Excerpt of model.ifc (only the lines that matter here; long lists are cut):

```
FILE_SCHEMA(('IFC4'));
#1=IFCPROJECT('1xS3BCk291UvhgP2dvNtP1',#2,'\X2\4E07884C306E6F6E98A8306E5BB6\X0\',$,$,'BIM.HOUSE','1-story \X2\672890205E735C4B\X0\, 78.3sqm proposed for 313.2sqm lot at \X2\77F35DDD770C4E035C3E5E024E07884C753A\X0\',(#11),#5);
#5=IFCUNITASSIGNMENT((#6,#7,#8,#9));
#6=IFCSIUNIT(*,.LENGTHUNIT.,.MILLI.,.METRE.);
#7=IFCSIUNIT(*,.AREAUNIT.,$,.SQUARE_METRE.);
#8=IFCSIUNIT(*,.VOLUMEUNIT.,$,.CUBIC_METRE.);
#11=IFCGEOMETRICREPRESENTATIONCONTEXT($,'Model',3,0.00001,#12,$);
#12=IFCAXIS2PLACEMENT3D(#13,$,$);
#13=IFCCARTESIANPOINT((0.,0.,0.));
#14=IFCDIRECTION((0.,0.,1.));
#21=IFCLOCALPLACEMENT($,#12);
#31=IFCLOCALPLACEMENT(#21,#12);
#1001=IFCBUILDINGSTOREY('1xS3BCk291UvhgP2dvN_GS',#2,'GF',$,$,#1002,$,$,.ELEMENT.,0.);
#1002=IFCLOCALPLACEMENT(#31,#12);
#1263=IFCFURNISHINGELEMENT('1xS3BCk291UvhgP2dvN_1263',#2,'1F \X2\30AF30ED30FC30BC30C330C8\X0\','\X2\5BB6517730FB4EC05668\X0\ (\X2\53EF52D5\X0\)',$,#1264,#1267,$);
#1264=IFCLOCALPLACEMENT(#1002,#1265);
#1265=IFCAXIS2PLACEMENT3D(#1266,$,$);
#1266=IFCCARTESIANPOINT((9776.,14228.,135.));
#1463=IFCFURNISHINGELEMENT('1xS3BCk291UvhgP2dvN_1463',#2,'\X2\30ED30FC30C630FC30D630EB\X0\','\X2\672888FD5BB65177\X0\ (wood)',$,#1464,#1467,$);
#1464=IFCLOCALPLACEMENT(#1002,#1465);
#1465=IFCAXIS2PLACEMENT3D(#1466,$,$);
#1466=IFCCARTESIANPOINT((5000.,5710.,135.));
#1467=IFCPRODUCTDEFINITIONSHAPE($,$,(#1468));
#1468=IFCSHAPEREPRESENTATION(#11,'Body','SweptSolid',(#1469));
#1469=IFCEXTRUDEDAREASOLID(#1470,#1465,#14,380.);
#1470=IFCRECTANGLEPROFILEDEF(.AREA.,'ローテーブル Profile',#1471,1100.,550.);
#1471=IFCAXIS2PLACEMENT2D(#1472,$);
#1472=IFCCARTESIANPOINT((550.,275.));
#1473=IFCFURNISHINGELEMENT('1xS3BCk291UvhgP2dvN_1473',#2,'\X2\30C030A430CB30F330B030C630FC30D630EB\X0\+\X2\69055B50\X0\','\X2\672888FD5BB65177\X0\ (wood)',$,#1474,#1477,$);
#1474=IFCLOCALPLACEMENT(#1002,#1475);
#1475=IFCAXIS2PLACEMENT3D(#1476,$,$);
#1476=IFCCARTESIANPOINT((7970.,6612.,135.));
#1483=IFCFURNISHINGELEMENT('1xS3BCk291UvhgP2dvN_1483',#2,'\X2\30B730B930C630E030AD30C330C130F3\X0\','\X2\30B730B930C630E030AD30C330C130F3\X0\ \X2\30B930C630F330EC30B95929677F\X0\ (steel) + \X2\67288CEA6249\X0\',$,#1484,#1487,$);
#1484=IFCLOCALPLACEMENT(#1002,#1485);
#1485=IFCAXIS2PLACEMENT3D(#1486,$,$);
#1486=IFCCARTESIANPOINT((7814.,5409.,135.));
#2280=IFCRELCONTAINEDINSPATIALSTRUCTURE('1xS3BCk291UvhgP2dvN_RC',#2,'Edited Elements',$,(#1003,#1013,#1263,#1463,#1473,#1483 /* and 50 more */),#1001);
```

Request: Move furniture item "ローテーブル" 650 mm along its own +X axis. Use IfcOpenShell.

```python
import ifcopenshell
import ifcopenshell.api.geometry
import ifcopenshell.util.placement

model = ifcopenshell.open("model.ifc")

item = model.by_guid("1xS3BCk291UvhgP2dvN_1463")
matrix = ifcopenshell.util.placement.get_local_placement(item.ObjectPlacement)
matrix[:3, 3] += matrix[:3, 0] * 650.0
ifcopenshell.api.geometry.edit_object_placement(model, product=item, matrix=matrix, is_si=False)

print(ifcopenshell.util.placement.get_local_placement(item.ObjectPlacement).round(3) + 0.0)

model.write("model-out.ifc")
```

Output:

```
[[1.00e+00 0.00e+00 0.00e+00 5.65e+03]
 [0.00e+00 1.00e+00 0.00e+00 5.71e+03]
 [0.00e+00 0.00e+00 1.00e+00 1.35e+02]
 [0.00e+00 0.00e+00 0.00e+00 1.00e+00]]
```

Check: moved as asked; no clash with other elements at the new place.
